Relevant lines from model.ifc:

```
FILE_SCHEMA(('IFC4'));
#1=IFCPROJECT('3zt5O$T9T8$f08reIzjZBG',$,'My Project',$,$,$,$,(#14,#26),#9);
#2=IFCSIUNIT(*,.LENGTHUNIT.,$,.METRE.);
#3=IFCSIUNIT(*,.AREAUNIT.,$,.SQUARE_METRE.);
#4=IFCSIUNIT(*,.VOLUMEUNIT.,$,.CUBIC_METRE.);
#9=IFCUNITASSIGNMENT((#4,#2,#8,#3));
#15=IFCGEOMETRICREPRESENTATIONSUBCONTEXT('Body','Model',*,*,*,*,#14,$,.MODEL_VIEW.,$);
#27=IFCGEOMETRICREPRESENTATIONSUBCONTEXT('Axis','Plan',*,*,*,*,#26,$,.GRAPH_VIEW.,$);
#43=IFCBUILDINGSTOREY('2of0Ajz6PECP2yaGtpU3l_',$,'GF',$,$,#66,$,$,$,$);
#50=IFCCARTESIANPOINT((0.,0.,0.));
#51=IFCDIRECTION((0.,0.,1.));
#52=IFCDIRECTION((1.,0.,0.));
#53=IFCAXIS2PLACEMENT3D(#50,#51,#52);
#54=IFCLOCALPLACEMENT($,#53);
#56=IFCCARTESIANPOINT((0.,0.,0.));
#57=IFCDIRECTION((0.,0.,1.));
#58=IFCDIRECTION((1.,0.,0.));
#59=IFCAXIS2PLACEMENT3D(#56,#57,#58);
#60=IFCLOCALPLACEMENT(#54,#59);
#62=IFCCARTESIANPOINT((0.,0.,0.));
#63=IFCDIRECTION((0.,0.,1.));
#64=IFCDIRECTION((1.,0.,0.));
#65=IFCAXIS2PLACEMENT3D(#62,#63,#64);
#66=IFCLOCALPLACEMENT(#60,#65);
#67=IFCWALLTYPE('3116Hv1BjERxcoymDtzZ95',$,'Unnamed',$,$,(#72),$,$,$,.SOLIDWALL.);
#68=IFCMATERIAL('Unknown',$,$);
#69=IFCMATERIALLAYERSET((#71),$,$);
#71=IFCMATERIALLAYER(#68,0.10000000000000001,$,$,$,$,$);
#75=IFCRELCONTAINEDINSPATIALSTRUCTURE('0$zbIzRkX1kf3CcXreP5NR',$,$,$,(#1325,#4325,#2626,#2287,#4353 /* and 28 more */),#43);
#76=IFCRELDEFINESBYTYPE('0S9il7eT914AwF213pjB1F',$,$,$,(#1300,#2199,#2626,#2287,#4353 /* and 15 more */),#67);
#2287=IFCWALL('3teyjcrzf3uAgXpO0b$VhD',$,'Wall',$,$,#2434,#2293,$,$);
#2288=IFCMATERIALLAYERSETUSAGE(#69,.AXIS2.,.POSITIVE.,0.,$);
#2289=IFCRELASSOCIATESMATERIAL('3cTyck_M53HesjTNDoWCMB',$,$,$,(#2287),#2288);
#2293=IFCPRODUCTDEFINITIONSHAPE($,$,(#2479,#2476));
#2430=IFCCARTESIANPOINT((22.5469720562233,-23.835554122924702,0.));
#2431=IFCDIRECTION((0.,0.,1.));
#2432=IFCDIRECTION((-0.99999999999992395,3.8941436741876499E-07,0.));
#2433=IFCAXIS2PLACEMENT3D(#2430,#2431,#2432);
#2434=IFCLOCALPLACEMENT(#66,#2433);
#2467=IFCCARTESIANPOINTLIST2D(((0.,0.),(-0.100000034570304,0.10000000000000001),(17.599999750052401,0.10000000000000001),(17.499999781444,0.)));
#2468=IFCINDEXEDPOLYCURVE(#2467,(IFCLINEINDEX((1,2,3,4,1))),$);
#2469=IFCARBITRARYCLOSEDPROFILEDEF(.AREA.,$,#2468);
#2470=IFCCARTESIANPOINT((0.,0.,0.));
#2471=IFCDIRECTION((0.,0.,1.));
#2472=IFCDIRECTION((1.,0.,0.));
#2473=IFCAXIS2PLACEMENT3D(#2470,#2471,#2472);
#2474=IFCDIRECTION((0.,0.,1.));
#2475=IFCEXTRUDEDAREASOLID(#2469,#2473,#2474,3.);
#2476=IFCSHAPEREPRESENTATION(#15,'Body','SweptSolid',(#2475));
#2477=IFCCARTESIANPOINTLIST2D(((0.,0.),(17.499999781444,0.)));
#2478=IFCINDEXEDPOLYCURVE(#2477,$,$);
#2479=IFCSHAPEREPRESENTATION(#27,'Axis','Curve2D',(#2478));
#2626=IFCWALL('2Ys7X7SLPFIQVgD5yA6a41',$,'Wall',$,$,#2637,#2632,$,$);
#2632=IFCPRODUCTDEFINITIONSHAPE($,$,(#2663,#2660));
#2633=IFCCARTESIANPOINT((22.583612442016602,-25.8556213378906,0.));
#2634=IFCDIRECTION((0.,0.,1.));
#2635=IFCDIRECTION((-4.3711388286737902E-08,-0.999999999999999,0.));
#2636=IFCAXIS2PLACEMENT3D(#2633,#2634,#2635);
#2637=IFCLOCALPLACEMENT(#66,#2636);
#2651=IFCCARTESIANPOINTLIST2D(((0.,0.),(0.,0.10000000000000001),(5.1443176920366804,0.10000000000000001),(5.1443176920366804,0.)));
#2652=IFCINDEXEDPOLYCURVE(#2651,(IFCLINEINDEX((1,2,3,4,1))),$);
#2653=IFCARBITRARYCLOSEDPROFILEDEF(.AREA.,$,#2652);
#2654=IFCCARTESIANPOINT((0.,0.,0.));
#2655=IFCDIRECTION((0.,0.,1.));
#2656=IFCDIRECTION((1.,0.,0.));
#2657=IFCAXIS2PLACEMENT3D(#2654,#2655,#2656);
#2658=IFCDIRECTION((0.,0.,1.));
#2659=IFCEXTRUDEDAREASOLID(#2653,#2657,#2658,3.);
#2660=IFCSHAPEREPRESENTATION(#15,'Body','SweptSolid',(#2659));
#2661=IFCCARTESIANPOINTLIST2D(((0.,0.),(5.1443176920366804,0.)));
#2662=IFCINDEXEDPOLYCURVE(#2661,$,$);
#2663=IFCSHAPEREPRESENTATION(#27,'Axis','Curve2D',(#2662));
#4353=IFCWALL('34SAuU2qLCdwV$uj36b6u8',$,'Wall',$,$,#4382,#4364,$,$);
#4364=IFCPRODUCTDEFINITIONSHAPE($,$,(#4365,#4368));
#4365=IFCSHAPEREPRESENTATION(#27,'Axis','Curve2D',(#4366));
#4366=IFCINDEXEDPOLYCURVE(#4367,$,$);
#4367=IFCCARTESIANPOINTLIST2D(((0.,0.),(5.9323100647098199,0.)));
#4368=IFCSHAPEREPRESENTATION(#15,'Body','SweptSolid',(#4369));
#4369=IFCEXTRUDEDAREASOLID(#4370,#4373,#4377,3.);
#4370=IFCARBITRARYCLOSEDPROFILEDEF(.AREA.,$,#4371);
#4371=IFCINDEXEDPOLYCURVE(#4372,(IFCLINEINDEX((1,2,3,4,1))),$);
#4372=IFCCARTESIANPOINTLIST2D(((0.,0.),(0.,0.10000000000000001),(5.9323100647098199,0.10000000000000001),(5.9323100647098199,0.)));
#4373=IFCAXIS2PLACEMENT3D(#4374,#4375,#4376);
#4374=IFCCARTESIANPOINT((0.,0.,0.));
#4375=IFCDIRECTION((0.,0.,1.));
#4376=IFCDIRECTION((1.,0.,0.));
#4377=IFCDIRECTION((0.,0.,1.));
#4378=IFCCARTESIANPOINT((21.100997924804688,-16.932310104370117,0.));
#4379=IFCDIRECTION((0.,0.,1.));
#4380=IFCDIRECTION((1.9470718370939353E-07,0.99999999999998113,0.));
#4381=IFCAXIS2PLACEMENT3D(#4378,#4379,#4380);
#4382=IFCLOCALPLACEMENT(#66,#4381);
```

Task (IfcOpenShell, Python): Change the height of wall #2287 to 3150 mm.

```python
import ifcopenshell
import ifcopenshell.geom
import ifcopenshell.util.representation
import ifcopenshell.util.shape
import ifcopenshell.util.unit

model = ifcopenshell.open("model.ifc")
unit_scale = ifcopenshell.util.unit.calculate_unit_scale(model)
settings = ifcopenshell.geom.settings()


def volume(element):
    """Net volume in cubic metres, openings subtracted."""
    shape = ifcopenshell.geom.create_shape(settings, element)
    return ifcopenshell.util.shape.get_volume(shape.geometry)


wall = model.by_guid("3teyjcrzf3uAgXpO0b$VhD")
before = volume(wall)

body = ifcopenshell.util.representation.get_representation(wall, "Model", "Body")
solid = body.Items[0]
old_height = solid.Depth
solid.Depth = 3.15 / unit_scale
after = volume(wall)

print(f"height {old_height:g} -> {solid.Depth:g}, volume {before:.3f} -> {after:.3f} m3")

model.write("model_edited.ifc")
```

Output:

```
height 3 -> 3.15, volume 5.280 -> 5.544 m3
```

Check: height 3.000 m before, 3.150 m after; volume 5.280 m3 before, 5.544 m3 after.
